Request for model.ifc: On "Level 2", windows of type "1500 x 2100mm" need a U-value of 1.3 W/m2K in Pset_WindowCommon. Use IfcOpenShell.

First a look at what the model holds.

```python
import ifcopenshell
import ifcopenshell.util.element

model = ifcopenshell.open("model.ifc")
print(model.schema)
storey = next(s for s in model.by_type("IfcBuildingStorey") if s.Name == "Level 2")
windows = [e for e in ifcopenshell.util.element.get_decomposition(storey) if e.is_a("IfcWindow")]
seen = {}
for e in windows:
    element_type = ifcopenshell.util.element.get_type(e)
    key = (element_type.Name if element_type != e and element_type else None, ifcopenshell.util.element.get_pset(e, "Pset_WindowCommon", "ThermalTransmittance"))
    seen[key] = seen.get(key, 0) + 1
for (name, value), count in sorted(seen.items(), key=str):
    print(count, "x", name, "|", value)
```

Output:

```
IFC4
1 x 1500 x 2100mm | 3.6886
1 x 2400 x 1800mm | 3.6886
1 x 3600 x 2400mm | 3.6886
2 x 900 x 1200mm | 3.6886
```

```python
import ifcopenshell
import ifcopenshell.api.pset
import ifcopenshell.util.element

model = ifcopenshell.open("model.ifc")

storey = next(s for s in model.by_type("IfcBuildingStorey") if s.Name == "Level 2")
windows = [e for e in ifcopenshell.util.element.get_decomposition(storey) if e.is_a("IfcWindow")]

count = 0
for e in windows:
    element_type = ifcopenshell.util.element.get_type(e)
    if element_type in (None, e) or element_type.Name != "1500 x 2100mm":
        continue
    # add_pset returns the element's existing set when there is one.
    pset = ifcopenshell.api.pset.add_pset(model, product=e, name="Pset_WindowCommon")
    ifcopenshell.api.pset.edit_pset(model, pset=pset, properties={"ThermalTransmittance": 1.3})
    count += 1

print(count, "windows updated")

model.write("model_v2.ifc")
```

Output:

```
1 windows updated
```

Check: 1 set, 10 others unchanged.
